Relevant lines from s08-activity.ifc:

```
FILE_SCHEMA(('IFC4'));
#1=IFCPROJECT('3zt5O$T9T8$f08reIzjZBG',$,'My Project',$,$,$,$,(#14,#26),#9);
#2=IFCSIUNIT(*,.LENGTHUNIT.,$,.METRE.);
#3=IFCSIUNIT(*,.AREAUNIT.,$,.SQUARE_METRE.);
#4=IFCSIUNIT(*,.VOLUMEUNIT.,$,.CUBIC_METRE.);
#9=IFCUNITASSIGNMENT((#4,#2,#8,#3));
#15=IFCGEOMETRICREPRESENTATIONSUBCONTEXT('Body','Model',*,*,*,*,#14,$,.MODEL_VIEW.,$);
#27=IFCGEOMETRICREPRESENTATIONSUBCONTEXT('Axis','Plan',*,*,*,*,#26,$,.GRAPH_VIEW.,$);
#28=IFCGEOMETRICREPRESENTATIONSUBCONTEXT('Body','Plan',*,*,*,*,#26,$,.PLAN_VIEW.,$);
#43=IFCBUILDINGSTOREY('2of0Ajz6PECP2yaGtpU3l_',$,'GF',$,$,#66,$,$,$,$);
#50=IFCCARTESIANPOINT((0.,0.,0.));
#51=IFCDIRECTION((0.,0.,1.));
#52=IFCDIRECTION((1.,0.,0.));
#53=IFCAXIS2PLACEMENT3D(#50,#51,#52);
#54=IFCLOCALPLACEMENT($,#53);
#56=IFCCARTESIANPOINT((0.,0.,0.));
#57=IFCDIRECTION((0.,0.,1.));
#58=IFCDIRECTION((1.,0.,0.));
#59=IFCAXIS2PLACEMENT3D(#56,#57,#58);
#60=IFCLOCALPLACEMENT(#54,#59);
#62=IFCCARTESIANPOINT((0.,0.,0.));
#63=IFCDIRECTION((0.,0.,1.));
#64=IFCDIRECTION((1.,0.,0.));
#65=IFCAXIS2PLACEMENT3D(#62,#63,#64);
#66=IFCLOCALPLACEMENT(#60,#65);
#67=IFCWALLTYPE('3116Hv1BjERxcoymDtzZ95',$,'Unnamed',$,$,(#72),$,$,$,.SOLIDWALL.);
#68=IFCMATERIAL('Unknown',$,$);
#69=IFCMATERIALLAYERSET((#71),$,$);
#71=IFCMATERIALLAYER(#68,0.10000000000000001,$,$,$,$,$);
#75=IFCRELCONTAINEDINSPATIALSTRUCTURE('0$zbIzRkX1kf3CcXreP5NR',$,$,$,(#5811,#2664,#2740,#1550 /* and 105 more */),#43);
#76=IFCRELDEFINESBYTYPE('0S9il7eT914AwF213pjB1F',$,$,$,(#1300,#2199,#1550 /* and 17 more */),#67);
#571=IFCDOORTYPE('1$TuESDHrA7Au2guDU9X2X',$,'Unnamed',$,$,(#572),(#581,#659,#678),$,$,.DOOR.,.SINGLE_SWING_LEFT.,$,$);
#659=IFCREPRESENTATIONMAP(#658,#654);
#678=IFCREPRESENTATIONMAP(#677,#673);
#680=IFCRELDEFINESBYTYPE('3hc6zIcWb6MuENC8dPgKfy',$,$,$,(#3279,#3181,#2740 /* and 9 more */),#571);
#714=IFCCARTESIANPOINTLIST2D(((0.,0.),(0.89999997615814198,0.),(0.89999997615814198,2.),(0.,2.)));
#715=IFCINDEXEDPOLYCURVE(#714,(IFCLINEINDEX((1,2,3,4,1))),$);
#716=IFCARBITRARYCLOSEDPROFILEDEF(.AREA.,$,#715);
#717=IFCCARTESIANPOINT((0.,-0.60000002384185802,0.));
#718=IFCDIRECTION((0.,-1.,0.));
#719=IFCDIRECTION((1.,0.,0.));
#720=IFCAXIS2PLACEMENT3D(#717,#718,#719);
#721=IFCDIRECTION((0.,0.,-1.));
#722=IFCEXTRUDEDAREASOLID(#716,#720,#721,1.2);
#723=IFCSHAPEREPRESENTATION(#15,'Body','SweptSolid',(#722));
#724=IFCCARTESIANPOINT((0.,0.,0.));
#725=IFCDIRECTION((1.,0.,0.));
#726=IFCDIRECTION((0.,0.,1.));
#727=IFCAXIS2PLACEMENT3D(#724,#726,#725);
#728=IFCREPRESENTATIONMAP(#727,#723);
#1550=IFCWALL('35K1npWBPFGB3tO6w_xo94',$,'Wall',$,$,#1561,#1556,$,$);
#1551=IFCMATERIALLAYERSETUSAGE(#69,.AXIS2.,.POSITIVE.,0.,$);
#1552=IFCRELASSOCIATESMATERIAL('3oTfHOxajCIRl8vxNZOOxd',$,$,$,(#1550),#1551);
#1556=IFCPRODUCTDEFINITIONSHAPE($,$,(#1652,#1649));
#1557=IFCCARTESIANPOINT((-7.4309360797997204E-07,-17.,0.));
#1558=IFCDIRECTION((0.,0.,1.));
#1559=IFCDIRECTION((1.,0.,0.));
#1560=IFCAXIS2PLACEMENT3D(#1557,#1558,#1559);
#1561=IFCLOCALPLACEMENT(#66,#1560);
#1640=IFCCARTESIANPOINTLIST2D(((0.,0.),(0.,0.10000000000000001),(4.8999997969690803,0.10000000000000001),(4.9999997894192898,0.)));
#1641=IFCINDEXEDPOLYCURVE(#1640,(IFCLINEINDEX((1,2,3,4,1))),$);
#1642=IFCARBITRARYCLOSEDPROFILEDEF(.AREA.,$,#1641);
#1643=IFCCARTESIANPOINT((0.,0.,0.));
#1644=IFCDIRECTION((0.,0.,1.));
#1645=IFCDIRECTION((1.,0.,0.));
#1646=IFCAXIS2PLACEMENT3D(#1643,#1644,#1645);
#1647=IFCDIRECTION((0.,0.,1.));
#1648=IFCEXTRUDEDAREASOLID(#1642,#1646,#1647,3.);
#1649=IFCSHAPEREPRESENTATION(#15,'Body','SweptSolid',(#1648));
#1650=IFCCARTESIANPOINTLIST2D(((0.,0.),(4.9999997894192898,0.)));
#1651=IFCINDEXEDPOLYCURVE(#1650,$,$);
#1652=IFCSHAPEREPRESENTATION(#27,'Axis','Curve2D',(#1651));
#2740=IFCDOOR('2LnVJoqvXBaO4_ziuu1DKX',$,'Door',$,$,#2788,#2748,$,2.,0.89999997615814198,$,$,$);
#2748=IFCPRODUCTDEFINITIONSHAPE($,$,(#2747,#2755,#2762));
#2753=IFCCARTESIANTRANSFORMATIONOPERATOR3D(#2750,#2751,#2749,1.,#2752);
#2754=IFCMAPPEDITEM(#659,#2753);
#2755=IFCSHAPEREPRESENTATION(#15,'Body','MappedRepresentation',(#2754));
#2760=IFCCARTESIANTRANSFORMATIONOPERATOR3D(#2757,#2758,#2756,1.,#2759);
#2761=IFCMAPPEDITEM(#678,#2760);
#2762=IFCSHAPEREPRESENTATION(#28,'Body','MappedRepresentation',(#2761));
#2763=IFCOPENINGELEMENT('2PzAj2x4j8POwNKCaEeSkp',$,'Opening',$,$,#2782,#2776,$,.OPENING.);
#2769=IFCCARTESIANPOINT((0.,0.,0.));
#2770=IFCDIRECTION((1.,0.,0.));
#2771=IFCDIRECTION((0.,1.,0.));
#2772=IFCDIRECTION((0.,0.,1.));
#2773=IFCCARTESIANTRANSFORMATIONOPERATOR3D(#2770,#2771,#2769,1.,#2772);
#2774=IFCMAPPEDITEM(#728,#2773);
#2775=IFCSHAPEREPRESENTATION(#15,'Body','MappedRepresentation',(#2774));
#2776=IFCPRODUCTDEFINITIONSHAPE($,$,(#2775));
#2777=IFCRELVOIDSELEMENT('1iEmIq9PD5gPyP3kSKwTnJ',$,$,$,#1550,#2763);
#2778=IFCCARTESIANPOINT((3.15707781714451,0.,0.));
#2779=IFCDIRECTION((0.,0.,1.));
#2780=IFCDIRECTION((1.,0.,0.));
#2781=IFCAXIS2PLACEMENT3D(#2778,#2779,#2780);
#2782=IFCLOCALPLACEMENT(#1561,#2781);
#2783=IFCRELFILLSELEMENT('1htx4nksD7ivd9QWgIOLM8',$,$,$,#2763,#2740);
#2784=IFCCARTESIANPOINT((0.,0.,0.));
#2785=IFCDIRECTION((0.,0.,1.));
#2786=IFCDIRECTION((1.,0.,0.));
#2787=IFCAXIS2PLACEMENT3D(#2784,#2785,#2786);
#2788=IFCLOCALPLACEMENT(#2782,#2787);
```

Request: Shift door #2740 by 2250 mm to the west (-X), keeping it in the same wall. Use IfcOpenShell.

```python
import ifcopenshell
import ifcopenshell.api.geometry
import ifcopenshell.util.placement

model = ifcopenshell.open("s08-activity.ifc")

door = model.by_guid("2LnVJoqvXBaO4_ziuu1DKX")
opening = door.FillsVoids[0].RelatingOpeningElement
wall = opening.VoidsElements[0].RelatingBuildingElement

wall_matrix = ifcopenshell.util.placement.get_local_placement(wall.ObjectPlacement)
shift = wall_matrix[:3, 0] * -2.25
before = ifcopenshell.util.placement.get_local_placement(door.ObjectPlacement)[:3, 3].copy()

# The door is placed relative to its opening, so it follows when the opening moves.
matrix = ifcopenshell.util.placement.get_local_placement(opening.ObjectPlacement)
matrix[:3, 3] += shift
ifcopenshell.api.geometry.edit_object_placement(
    model, product=opening, matrix=matrix, is_si=False, should_transform_children=True
)

after = ifcopenshell.util.placement.get_local_placement(door.ObjectPlacement)[:3, 3]
print("door moved by", (after - before).round(3) + 0.0)

model.write("s08-activity_v2.ifc")
```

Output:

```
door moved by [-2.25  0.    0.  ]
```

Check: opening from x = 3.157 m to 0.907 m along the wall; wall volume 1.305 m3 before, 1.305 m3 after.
